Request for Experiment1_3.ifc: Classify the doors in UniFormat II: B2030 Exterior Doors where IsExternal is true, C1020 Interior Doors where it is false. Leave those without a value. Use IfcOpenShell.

First a look at what the model holds.

```python
import ifcopenshell
import ifcopenshell.util.element

model = ifcopenshell.open("Experiment1_3.ifc")
print(model.schema)
print("classifications:", [c.Name for c in model.by_type("IfcClassification")])
values = [ifcopenshell.util.element.get_pset(e, "Pset_DoorCommon", "IsExternal") for e in model.by_type("IfcDoor")]
for value in (True, False, None):
    print("IsExternal", value, values.count(value))
```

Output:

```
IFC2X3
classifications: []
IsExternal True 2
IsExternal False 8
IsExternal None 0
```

```python
import ifcopenshell
import ifcopenshell.api.classification
import ifcopenshell.util.element

model = ifcopenshell.open("Experiment1_3.ifc")

# IFC2X3 requires Source and Edition and has no link from the project to the system.
system = model.create_entity("IfcClassification", Source="ASTM", Edition="E1557", Name="UniFormat II")

doors = model.by_type("IfcDoor")
external = {e: ifcopenshell.util.element.get_pset(e, "Pset_DoorCommon", "IsExternal") for e in doors}
for flag, code, name in ((True, "B2030", "Exterior Doors"), (False, "C1020", "Interior Doors")):
    products = [e for e in doors if external[e] is flag]
    ifcopenshell.api.classification.add_reference(
        model, products=products, classification=system, identification=code, name=name
    )
    print(code, len(products))

model.write("Experiment1_3_updated.ifc")
```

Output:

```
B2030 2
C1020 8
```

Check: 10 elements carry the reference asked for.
